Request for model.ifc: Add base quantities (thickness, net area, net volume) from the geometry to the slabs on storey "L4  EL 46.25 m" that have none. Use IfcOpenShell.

First a look at what the model holds.

```python
import ifcopenshell
import ifcopenshell.util.element
import ifcopenshell.util.unit

model = ifcopenshell.open("model.ifc")
print(model.schema)
for unit_type in ("LENGTHUNIT", "AREAUNIT", "VOLUMEUNIT"):
    print(unit_type, ifcopenshell.util.unit.calculate_unit_scale(model, unit_type))
storey = next(s for s in model.by_type("IfcBuildingStorey") if s.Name == "L4  EL 46.25 m")
slabs = [e for e in ifcopenshell.util.element.get_decomposition(storey) if e.is_a("IfcSlab")]
for e in sorted(slabs, key=lambda e: e.id()):
    print(e.id(), e.is_a(), e.Name, list(ifcopenshell.util.element.get_psets(e, qtos_only=True)), sep=" | ")
```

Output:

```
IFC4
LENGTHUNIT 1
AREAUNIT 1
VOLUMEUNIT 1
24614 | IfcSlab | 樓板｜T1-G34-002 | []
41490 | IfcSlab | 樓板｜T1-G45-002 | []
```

```python
import ifcopenshell
import ifcopenshell.api.pset
import ifcopenshell.geom
import ifcopenshell.util.element
import ifcopenshell.util.shape
import ifcopenshell.util.unit

model = ifcopenshell.open("model.ifc")
unit_scale = ifcopenshell.util.unit.calculate_unit_scale(model)
area_scale = ifcopenshell.util.unit.calculate_unit_scale(model, "AREAUNIT")
volume_scale = ifcopenshell.util.unit.calculate_unit_scale(model, "VOLUMEUNIT")
settings = ifcopenshell.geom.settings()

storey = next(s for s in model.by_type("IfcBuildingStorey") if s.Name == "L4  EL 46.25 m")
slabs = [e for e in ifcopenshell.util.element.get_decomposition(storey) if e.is_a("IfcSlab")]

for e in sorted(slabs, key=lambda e: e.id()):
    if ifcopenshell.util.element.get_psets(e, qtos_only=True, should_inherit=False):
        continue
    # Geometry comes back in metres, in the element's own axes.
    shape = ifcopenshell.geom.create_shape(settings, e)
    values = {
        "Width": ifcopenshell.util.shape.get_z(shape.geometry) / unit_scale,
        "NetArea": ifcopenshell.util.shape.get_footprint_area(shape.geometry) / area_scale,
        "NetVolume": ifcopenshell.util.shape.get_volume(shape.geometry) / volume_scale,
    }
    qto = ifcopenshell.api.pset.add_qto(model, product=e, name="Qto_SlabBaseQuantities")
    ifcopenshell.api.pset.edit_qto(model, qto=qto, properties=values)
    print(e.id(), {k: round(v, 3) for k, v in values.items()})

model.write("model_updated.ifc")
```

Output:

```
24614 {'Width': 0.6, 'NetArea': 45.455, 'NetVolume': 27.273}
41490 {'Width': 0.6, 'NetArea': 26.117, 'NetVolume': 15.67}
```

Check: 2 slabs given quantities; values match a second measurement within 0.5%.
